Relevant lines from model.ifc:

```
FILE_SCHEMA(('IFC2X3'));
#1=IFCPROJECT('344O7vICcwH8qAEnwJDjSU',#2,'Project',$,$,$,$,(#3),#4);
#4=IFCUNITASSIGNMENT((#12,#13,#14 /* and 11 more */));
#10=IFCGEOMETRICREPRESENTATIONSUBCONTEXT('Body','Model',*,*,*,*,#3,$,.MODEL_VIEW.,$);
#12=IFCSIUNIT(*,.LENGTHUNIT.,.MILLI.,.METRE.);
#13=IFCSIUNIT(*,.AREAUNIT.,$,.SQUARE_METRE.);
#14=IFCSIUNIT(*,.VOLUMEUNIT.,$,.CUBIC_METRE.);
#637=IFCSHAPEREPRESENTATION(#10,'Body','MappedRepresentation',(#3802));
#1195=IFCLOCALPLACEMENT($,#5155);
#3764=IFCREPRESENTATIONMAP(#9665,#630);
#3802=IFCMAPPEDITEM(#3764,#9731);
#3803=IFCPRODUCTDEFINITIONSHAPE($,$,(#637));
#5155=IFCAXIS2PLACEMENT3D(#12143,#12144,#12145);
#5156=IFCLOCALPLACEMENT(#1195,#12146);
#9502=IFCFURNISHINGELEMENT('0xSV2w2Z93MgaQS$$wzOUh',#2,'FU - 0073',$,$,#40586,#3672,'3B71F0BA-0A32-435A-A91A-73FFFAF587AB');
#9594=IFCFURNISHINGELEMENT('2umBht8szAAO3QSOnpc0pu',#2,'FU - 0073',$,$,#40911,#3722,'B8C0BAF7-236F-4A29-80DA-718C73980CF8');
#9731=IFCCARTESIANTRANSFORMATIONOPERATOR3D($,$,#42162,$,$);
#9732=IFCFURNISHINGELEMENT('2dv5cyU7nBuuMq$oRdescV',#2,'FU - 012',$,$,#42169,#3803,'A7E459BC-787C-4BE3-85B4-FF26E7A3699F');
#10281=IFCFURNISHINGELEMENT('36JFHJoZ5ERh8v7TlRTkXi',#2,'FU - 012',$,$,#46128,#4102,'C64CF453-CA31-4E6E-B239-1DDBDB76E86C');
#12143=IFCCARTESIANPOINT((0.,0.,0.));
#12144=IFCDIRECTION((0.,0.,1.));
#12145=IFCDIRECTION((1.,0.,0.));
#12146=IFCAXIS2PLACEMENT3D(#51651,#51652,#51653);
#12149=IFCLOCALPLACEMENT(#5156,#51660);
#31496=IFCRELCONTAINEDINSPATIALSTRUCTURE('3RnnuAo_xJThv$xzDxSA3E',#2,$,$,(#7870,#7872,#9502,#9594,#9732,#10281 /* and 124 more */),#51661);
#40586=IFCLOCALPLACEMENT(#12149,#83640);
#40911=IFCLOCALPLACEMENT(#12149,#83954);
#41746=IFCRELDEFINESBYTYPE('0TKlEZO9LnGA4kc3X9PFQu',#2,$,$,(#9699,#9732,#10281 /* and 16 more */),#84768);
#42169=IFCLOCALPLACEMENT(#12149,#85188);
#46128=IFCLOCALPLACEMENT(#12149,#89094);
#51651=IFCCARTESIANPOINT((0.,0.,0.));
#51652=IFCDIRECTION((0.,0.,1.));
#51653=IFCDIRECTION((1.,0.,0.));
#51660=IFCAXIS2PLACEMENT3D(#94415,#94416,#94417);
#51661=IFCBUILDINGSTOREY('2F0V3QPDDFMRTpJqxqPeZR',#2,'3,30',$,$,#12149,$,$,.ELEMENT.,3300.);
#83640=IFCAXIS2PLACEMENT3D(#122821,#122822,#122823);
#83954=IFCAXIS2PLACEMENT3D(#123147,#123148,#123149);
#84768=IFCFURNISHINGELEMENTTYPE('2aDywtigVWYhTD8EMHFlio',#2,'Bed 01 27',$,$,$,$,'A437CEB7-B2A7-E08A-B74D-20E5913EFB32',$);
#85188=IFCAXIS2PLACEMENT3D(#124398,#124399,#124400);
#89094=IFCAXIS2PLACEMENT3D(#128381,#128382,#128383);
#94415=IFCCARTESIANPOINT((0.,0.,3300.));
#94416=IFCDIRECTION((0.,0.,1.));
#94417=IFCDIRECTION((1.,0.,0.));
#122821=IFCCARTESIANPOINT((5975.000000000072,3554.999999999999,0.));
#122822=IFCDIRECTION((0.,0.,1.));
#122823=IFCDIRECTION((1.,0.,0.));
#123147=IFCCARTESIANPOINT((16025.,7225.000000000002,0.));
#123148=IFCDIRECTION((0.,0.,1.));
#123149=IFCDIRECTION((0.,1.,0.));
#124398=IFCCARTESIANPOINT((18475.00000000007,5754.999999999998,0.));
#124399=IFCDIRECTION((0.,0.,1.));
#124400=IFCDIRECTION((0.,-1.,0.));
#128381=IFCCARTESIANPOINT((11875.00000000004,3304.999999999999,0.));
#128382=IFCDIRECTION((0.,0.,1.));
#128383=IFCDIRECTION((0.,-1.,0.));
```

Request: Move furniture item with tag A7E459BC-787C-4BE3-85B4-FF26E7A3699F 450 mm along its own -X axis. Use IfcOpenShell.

```python
import ifcopenshell
import ifcopenshell.api.geometry
import ifcopenshell.util.placement

model = ifcopenshell.open("model.ifc")

item = model.by_id(9732)
matrix = ifcopenshell.util.placement.get_local_placement(item.ObjectPlacement)
matrix[:3, 3] -= matrix[:3, 0] * 450.0
ifcopenshell.api.geometry.edit_object_placement(model, product=item, matrix=matrix, is_si=False)

print(ifcopenshell.util.placement.get_local_placement(item.ObjectPlacement).round(3) + 0.0)

model.write("model_updated.ifc")
```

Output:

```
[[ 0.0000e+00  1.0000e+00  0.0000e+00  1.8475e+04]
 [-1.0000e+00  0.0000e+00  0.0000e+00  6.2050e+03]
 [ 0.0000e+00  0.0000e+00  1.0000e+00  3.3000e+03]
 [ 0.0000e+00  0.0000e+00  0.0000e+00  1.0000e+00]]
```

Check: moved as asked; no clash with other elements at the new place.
